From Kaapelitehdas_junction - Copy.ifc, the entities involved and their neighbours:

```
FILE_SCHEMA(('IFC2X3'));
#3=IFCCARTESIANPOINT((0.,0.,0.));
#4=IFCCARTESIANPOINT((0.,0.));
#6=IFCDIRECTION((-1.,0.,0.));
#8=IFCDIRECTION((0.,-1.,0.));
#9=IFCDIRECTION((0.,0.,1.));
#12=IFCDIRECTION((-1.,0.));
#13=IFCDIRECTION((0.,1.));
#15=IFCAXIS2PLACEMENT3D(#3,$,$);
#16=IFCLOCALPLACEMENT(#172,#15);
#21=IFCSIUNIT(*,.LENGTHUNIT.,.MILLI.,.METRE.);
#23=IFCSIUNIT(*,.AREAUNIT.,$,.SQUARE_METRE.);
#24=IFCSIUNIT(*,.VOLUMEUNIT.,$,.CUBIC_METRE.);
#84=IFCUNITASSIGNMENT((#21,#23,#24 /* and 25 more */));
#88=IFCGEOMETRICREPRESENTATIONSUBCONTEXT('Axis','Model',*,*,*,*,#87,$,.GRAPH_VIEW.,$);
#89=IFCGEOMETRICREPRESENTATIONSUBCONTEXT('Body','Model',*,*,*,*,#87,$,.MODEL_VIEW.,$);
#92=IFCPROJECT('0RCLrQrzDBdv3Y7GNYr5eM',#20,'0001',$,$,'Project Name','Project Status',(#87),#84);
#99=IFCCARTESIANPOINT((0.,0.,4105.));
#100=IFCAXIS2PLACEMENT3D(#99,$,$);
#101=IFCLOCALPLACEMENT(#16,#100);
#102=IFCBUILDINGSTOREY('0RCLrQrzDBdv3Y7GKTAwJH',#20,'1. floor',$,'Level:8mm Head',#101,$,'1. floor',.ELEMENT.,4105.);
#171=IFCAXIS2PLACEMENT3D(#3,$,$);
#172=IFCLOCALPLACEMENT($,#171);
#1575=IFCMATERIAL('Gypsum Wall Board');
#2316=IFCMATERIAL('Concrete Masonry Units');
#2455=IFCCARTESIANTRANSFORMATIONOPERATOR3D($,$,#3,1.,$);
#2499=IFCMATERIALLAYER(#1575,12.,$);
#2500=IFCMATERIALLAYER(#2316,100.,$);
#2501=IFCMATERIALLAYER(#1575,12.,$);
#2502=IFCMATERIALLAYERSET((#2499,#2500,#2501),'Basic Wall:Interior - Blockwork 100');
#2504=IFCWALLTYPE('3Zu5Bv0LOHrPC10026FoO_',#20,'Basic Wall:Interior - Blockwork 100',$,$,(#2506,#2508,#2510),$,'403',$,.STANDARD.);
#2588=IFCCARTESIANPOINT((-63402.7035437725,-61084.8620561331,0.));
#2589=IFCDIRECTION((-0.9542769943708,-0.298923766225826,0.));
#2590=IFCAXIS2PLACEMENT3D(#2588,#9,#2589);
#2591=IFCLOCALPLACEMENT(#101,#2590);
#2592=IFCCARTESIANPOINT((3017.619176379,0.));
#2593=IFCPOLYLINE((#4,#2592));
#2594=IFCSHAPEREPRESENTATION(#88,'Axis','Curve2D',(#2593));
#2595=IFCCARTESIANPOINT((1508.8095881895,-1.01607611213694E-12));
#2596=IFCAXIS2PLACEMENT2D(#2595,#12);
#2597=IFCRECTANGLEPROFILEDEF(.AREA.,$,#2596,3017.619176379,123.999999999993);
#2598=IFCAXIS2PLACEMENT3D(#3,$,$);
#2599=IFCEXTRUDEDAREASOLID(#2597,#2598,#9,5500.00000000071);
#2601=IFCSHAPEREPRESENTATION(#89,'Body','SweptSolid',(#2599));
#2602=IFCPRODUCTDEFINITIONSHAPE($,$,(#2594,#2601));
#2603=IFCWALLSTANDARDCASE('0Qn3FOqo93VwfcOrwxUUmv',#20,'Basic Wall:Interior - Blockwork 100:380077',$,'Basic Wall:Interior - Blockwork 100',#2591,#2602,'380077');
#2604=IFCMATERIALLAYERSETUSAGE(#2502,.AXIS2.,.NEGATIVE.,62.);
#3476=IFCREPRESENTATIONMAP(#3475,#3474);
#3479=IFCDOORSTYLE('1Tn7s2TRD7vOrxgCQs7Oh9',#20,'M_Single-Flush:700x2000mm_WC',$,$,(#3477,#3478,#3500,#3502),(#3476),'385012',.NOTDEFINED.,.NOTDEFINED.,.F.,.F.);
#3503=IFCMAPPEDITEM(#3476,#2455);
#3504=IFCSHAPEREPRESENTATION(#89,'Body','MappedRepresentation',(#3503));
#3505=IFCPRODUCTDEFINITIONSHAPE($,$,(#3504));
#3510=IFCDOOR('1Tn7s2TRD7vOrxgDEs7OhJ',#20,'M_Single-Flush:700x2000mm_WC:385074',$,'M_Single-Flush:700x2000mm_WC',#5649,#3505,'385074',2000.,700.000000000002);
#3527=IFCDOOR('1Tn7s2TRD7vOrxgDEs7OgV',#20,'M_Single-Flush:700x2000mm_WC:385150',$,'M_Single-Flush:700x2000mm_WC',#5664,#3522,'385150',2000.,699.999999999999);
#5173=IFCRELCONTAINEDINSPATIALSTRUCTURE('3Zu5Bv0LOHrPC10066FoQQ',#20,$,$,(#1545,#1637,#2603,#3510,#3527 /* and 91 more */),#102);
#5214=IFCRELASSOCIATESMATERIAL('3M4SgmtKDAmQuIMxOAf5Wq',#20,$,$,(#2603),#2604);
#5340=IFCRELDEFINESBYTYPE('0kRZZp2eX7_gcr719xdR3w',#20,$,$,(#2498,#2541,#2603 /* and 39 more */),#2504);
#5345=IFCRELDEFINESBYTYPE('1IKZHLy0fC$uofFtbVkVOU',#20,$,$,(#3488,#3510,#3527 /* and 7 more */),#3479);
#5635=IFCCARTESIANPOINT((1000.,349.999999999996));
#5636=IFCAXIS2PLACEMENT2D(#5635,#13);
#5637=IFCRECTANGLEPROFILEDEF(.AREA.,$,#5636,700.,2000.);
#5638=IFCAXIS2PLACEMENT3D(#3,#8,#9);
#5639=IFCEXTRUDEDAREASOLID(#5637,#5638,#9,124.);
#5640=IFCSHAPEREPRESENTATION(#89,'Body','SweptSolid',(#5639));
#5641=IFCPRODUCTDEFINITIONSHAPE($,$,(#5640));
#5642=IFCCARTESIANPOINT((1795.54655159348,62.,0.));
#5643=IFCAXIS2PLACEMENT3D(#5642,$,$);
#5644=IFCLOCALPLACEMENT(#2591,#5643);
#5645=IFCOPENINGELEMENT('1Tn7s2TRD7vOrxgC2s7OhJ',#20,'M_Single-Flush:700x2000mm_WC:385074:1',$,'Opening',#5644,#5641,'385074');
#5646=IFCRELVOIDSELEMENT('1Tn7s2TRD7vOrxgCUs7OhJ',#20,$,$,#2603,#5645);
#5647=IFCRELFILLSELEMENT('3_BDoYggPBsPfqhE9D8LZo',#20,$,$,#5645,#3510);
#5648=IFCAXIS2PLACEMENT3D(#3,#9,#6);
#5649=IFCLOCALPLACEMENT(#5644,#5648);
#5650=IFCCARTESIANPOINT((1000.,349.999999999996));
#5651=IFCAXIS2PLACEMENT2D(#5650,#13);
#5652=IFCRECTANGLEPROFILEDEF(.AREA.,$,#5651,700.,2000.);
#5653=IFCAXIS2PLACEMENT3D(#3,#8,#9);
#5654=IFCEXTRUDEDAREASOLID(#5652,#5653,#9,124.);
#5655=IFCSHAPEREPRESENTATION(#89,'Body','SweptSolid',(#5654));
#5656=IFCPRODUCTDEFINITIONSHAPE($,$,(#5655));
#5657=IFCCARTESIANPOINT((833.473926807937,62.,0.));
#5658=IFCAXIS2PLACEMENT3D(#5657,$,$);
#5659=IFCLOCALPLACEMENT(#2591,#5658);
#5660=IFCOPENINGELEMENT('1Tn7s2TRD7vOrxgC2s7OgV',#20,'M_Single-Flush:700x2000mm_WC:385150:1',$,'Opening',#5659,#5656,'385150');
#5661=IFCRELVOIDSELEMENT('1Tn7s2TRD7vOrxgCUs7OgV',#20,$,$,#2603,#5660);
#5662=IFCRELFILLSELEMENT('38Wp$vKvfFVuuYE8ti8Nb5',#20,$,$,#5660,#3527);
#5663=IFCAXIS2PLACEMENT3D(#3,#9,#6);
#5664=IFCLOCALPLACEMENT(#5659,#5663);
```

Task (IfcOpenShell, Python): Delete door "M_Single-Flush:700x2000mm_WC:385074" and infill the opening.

```python
import ifcopenshell
import ifcopenshell.api.feature
import ifcopenshell.api.root
import ifcopenshell.geom
import ifcopenshell.util.shape

model = ifcopenshell.open("Kaapelitehdas_junction - Copy.ifc")
settings = ifcopenshell.geom.settings()


def volume(element):
    """Net volume in cubic metres, openings subtracted."""
    shape = ifcopenshell.geom.create_shape(settings, element)
    return ifcopenshell.util.shape.get_volume(shape.geometry)


door = model.by_guid("1Tn7s2TRD7vOrxgDEs7OhJ")
opening = door.FillsVoids[0].RelatingOpeningElement
wall = opening.VoidsElements[0].RelatingBuildingElement
before = volume(wall)

ifcopenshell.api.root.remove_product(model, product=door)
ifcopenshell.api.feature.remove_feature(model, feature=opening)

after = volume(wall)

print(f"wall volume {before:.3f} -> {after:.3f} m3")

model.write("Kaapelitehdas_junction - Copy_edited.ifc")
```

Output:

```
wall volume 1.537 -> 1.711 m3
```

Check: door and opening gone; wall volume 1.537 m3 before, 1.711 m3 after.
